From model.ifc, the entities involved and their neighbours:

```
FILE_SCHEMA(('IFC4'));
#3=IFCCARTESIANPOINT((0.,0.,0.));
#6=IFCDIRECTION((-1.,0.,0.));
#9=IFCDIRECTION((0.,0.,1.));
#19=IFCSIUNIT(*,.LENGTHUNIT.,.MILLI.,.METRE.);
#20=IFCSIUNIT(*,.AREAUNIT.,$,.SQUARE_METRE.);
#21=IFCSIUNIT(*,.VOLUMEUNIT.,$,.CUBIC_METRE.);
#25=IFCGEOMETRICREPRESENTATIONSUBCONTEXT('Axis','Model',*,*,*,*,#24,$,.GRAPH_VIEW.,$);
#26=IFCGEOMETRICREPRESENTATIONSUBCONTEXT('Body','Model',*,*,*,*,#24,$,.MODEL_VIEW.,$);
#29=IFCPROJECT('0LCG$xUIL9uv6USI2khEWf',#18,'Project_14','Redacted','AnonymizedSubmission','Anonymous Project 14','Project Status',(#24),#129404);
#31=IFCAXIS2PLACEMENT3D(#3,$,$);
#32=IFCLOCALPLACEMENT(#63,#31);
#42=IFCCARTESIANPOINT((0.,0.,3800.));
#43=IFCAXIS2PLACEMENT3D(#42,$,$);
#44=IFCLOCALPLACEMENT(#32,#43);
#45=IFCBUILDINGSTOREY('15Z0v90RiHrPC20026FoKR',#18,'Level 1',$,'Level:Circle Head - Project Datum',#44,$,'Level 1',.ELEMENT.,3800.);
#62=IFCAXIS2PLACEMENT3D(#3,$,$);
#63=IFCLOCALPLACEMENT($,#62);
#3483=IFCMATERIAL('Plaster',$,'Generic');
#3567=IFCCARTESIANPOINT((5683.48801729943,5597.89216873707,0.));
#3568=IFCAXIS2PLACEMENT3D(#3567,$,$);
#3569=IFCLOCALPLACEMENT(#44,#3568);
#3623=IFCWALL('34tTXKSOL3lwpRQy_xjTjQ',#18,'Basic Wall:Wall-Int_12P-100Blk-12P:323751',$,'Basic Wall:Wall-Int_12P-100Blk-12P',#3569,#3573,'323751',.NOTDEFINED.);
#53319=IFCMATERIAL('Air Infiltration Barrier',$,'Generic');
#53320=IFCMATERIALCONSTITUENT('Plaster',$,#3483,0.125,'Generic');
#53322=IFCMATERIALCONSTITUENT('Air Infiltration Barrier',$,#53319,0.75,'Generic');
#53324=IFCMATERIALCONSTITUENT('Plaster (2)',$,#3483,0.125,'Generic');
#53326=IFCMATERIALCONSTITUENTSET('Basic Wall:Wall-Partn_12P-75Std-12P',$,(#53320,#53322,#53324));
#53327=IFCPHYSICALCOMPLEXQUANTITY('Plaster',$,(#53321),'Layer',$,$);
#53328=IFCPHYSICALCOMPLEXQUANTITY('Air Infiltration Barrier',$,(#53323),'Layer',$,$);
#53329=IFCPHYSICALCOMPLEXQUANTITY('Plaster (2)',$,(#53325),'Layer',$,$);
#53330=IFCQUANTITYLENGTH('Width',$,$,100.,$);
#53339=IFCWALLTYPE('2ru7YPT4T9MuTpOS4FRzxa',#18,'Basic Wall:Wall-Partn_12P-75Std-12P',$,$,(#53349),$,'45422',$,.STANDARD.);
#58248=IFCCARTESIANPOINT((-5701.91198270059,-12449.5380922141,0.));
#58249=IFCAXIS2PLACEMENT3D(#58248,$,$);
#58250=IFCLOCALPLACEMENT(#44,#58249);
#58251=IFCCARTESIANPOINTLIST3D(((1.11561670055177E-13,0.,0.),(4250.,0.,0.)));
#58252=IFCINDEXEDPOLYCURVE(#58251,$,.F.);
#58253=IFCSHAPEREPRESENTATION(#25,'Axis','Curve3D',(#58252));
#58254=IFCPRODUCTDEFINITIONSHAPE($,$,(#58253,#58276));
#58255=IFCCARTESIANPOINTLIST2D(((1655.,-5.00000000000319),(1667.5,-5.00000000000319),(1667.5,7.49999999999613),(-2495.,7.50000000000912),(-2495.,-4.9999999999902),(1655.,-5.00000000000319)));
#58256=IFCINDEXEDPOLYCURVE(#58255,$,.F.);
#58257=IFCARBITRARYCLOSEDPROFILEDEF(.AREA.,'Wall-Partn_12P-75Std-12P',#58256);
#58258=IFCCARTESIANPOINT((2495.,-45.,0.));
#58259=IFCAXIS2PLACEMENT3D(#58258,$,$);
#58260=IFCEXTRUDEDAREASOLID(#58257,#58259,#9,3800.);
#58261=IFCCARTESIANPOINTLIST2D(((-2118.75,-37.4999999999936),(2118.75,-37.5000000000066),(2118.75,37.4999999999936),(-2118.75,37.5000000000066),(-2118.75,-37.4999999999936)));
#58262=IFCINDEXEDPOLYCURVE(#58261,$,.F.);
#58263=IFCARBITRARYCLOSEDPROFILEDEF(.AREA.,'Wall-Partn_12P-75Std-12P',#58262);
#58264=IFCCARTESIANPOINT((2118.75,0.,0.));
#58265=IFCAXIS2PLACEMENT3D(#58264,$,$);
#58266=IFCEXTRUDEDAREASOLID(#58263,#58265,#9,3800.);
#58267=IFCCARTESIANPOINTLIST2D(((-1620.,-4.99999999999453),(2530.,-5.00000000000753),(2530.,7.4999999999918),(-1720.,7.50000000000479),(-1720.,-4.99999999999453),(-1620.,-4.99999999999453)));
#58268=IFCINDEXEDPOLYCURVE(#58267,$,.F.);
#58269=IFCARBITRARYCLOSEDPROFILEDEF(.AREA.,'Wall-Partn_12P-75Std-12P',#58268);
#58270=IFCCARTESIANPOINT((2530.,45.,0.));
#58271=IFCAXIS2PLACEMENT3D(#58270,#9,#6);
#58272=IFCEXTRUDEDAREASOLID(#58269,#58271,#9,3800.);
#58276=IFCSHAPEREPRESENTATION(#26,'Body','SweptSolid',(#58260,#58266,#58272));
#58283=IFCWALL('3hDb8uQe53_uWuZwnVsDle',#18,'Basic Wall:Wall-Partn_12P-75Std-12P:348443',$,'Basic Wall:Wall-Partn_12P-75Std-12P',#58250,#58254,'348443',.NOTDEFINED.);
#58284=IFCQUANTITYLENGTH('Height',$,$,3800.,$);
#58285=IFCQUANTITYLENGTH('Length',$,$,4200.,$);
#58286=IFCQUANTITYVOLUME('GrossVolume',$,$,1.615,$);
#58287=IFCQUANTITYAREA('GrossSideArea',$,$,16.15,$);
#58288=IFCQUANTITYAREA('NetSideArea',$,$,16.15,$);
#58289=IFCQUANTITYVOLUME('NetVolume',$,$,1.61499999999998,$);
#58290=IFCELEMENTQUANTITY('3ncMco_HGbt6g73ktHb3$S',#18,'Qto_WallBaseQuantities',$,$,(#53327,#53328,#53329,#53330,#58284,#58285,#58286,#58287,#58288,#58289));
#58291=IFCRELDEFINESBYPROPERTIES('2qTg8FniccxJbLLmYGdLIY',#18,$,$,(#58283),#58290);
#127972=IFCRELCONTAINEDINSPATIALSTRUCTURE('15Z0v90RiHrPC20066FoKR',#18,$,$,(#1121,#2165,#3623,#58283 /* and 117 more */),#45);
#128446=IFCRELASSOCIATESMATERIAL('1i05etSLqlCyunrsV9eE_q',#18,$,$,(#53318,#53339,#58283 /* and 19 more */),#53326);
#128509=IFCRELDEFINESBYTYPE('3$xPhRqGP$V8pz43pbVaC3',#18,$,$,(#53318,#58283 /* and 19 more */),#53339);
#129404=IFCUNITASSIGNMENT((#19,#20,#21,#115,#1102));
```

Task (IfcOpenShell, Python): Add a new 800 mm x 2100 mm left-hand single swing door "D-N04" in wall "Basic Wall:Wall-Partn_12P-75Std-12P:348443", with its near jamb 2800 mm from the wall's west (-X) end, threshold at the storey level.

```python
import numpy as np
import ifcopenshell
import ifcopenshell.api.feature
import ifcopenshell.api.geometry
import ifcopenshell.api.pset
import ifcopenshell.api.root
import ifcopenshell.api.spatial
import ifcopenshell.geom
import ifcopenshell.util.element
import ifcopenshell.util.placement
import ifcopenshell.util.representation
import ifcopenshell.util.shape
import ifcopenshell.util.unit

model = ifcopenshell.open("model.ifc")
unit_scale = ifcopenshell.util.unit.calculate_unit_scale(model)
area_scale = ifcopenshell.util.unit.calculate_unit_scale(model, "AREAUNIT")
volume_scale = ifcopenshell.util.unit.calculate_unit_scale(model, "VOLUMEUNIT")
settings = ifcopenshell.geom.settings()


def volume(element):
    """Net volume in cubic metres, openings subtracted."""
    shape = ifcopenshell.geom.create_shape(settings, element)
    return ifcopenshell.util.shape.get_volume(shape.geometry)


wall = model.by_guid("3hDb8uQe53_uWuZwnVsDle")
storey = ifcopenshell.util.element.get_container(wall, ifc_class="IfcBuildingStorey")
context = ifcopenshell.util.representation.get_context(model, "Model", "Body", "MODEL_VIEW")
before = volume(wall)

width, height, from_end, sill = 0.8, 2.1, 2.8, 0.0  # metres

# The wall runs along its own X axis, and the end named is its -X end.
wall_shape = ifcopenshell.geom.create_shape(settings, wall)
x, y, z = ifcopenshell.util.shape.get_vertices(wall_shape.geometry).T
start = x.min() + from_end
face, thickness = float(y.min()), float(y.max() - y.min())
wall_matrix = ifcopenshell.util.placement.get_local_placement(wall.ObjectPlacement)
level = ifcopenshell.util.placement.get_local_placement(storey.ObjectPlacement)[2, 3]


def in_wall(x, y):
    """Placement at x, y metres in the wall's axes, at sill height."""
    matrix = wall_matrix.copy()
    matrix[:, 3] = wall_matrix @ np.array([x / unit_scale, y / unit_scale, 0.0, 1.0])
    matrix[2, 3] = level + sill / unit_scale
    return matrix


# Opening: a box that overshoots both wall faces by 50 mm.
opening = ifcopenshell.api.root.create_entity(model, ifc_class="IfcOpeningElement", predefined_type="OPENING")
box = ifcopenshell.api.geometry.add_wall_representation(
    model, context=context, length=width, height=height, thickness=thickness + 0.1
)
ifcopenshell.api.geometry.assign_representation(model, product=opening, representation=box)
ifcopenshell.api.geometry.edit_object_placement(model, product=opening, matrix=in_wall(start, face - 0.05), is_si=False)
ifcopenshell.api.feature.add_feature(model, feature=opening, element=wall)

door = ifcopenshell.api.root.create_entity(model, ifc_class="IfcDoor", name="D-N04", predefined_type="DOOR")
door.OverallWidth, door.OverallHeight = width / unit_scale, height / unit_scale
door.OperationType = "SINGLE_SWING_LEFT"
body = ifcopenshell.api.geometry.add_door_representation(
    model,
    context=context,
    overall_width=door.OverallWidth,
    overall_height=door.OverallHeight,
    operation_type="SINGLE_SWING_LEFT",
    lining_properties={"LiningDepth": thickness / unit_scale, "ThresholdDepth": thickness / unit_scale},
)
ifcopenshell.api.geometry.assign_representation(model, product=door, representation=body)
ifcopenshell.api.spatial.assign_container(model, products=[door], relating_structure=storey)
ifcopenshell.api.feature.add_filling(model, opening=opening, element=door)

# The lining spans the wall, so the door starts at the wall face.
ifcopenshell.api.geometry.edit_object_placement(model, product=door, matrix=in_wall(start, face), is_si=False)

after = volume(wall)

# Update the wall's stored quantities.
qto = model.by_id(ifcopenshell.util.element.get_pset(wall, "Qto_WallBaseQuantities", should_inherit=False)["id"])
ifcopenshell.api.pset.edit_qto(model, qto=qto, properties={
    "NetSideArea": after / thickness / area_scale,
    "NetVolume": after / volume_scale,
})

print(f"wall volume {before:.3f} -> {after:.3f} m3")

model.write("model-out.ifc")
```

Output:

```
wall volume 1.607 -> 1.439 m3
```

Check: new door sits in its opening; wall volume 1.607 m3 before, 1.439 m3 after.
